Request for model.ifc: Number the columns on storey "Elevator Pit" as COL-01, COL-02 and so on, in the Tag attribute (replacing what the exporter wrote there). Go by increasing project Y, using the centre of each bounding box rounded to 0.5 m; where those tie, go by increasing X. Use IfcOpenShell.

First a look at what the model holds.

```python
import ifcopenshell
import ifcopenshell.util.element
import ifcopenshell.util.placement

model = ifcopenshell.open("model.ifc")
print(model.schema)
storey = next(s for s in model.by_type("IfcBuildingStorey") if s.Name == "Elevator Pit")
columns = [e for e in ifcopenshell.util.element.get_decomposition(storey) if e.is_a("IfcColumn")]
for e in sorted(columns, key=lambda e: e.id()):
    origin = ifcopenshell.util.placement.get_local_placement(e.ObjectPlacement)[:3, 3]
    print(e.id(), e.Tag, e.Name, origin.round(2) + 0.0, sep=" | ")
```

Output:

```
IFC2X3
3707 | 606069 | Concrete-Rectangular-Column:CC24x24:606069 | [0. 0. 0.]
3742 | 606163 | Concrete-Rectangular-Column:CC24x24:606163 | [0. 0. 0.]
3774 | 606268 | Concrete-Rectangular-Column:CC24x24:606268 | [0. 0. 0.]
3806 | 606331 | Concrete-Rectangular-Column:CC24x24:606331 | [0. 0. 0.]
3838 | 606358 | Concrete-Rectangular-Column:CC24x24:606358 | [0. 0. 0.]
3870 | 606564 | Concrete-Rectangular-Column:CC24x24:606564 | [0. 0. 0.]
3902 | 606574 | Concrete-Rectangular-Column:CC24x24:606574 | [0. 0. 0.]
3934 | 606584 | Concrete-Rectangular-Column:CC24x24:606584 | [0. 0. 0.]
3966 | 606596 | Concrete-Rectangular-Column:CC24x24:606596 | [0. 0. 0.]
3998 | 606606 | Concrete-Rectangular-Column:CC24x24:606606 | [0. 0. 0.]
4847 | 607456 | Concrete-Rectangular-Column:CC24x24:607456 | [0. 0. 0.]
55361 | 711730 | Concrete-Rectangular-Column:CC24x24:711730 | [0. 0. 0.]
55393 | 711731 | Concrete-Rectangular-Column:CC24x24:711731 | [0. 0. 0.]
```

```python
import ifcopenshell
import ifcopenshell.geom
import ifcopenshell.util.element
import ifcopenshell.util.shape

model = ifcopenshell.open("model.ifc")
settings = ifcopenshell.geom.settings()
settings.set("use-world-coords", True)


def centre(element):
    shape = ifcopenshell.geom.create_shape(settings, element)
    return ifcopenshell.util.shape.get_bbox_centroid(shape.geometry)


storey = next(s for s in model.by_type("IfcBuildingStorey") if s.Name == "Elevator Pit")
columns = [e for e in ifcopenshell.util.element.get_decomposition(storey) if e.is_a("IfcColumn")]

# Insertion points can sit at a corner or the storey origin, so sort by the geometry (in metres).
centres = {e: centre(e) for e in columns}
columns.sort(key=lambda e: (round(centres[e][1] / 0.5), centres[e][0]))

for i, e in enumerate(columns, start=1):
    number = f"COL-{i:02d}"
    e.Tag = number
    print(e.id(), number)

model.write("model-out.ifc")
```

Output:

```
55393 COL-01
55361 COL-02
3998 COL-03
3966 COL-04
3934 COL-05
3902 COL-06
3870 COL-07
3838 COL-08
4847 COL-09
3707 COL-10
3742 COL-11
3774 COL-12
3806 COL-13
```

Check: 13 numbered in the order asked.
